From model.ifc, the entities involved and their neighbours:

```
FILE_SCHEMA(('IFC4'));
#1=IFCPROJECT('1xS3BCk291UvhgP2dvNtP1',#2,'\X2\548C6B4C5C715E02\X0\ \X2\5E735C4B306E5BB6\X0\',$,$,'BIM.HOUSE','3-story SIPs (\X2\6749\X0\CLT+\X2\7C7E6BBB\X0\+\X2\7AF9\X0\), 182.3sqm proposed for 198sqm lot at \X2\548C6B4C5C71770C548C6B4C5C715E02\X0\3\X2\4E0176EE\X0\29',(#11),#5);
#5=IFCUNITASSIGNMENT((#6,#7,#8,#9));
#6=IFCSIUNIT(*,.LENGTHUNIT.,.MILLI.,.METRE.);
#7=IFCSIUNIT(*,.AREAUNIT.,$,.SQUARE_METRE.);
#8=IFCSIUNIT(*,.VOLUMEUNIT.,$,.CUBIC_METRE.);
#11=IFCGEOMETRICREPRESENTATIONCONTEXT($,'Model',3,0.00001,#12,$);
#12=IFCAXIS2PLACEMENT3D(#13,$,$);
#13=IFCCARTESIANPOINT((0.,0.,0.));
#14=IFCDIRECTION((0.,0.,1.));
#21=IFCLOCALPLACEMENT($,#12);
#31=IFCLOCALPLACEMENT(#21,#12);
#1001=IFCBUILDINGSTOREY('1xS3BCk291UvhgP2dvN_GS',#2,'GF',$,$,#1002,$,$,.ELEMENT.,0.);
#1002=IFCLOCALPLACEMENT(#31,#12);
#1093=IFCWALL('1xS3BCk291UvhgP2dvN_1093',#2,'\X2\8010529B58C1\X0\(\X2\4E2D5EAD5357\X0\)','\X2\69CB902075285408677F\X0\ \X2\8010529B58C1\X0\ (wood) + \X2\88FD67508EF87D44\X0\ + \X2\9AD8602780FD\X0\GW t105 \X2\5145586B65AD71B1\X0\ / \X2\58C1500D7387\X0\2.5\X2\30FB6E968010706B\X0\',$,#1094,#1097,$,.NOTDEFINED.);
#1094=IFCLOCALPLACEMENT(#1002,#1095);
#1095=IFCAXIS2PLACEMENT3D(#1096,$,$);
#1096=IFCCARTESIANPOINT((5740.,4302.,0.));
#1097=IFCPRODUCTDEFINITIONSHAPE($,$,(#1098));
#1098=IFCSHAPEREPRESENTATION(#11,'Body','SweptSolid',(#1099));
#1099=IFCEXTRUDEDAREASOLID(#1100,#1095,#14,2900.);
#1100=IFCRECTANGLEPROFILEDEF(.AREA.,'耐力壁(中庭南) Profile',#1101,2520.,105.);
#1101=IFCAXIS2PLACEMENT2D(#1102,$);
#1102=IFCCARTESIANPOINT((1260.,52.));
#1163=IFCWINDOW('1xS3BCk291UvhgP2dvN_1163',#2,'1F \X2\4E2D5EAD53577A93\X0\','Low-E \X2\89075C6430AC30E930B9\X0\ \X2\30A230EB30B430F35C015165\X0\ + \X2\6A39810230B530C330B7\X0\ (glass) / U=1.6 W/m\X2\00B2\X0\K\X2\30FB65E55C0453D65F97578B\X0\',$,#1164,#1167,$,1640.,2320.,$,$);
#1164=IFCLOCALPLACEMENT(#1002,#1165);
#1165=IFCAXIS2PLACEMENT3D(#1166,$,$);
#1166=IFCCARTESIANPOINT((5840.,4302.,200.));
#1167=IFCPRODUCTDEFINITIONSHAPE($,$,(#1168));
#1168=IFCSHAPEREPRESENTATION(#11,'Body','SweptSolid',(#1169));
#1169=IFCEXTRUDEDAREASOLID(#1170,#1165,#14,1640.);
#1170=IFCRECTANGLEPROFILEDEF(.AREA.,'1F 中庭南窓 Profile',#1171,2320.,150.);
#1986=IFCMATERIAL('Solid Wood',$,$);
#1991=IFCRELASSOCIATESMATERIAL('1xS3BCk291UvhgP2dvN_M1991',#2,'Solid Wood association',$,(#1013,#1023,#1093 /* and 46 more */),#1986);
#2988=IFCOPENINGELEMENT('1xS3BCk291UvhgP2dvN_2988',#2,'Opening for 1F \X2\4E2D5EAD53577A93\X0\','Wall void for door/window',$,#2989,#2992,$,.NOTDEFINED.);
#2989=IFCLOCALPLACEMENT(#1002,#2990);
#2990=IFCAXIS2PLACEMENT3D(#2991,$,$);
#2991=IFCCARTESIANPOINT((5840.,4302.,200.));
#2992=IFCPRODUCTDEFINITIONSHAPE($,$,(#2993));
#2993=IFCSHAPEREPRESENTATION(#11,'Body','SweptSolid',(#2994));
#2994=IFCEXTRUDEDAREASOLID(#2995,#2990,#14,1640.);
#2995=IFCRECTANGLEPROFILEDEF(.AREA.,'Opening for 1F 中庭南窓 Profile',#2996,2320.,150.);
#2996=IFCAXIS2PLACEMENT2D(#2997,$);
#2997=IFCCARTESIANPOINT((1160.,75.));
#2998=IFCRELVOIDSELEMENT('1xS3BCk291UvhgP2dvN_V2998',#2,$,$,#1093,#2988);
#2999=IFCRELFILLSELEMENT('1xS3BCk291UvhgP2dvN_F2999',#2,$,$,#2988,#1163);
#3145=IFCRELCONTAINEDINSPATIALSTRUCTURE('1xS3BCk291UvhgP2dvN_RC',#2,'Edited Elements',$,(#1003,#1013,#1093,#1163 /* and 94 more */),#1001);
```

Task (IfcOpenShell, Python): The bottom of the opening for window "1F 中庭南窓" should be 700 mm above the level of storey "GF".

```python
import numpy as np
import ifcopenshell
import ifcopenshell.api.geometry
import ifcopenshell.geom
import ifcopenshell.util.element
import ifcopenshell.util.placement
import ifcopenshell.util.shape
import ifcopenshell.util.unit

model = ifcopenshell.open("model.ifc")
unit_scale = ifcopenshell.util.unit.calculate_unit_scale(model)

window = model.by_guid("1xS3BCk291UvhgP2dvN_1163")
opening = window.FillsVoids[0].RelatingOpeningElement
storey = ifcopenshell.util.element.get_container(window, ifc_class="IfcBuildingStorey")
level = ifcopenshell.util.placement.get_local_placement(storey.ObjectPlacement)[2, 3]

# The opening's origin need not be at the sill, so measure its lowest point.
shape = ifcopenshell.geom.create_shape(ifcopenshell.geom.settings(), opening)
bottom = ifcopenshell.util.shape.get_shape_bottom_elevation(shape, shape.geometry) / unit_scale
dz = level + 700.0 - bottom

shift = np.array([0.0, 0.0, dz])
# The window is not placed relative to its opening, so move both.
for product in (opening, window):
    matrix = ifcopenshell.util.placement.get_local_placement(product.ObjectPlacement)
    matrix[:3, 3] += shift
    ifcopenshell.api.geometry.edit_object_placement(model, product=product, matrix=matrix, is_si=False)

print(f"moved by {dz * unit_scale:+.3f} m")

model.write("model-out.ifc")
```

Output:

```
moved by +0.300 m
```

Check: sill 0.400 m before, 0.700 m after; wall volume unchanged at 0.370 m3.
